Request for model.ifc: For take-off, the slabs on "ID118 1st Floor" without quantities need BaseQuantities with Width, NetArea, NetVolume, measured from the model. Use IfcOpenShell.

First a look at what the model holds.

```python
import ifcopenshell
import ifcopenshell.util.element
import ifcopenshell.util.unit

model = ifcopenshell.open("model.ifc")
print(model.schema)
for unit_type in ("LENGTHUNIT", "AREAUNIT", "VOLUMEUNIT"):
    print(unit_type, ifcopenshell.util.unit.calculate_unit_scale(model, unit_type))
storey = next(s for s in model.by_type("IfcBuildingStorey") if s.Name == "ID118 1st Floor")
slabs = [e for e in ifcopenshell.util.element.get_decomposition(storey) if e.is_a("IfcSlab")]
for e in sorted(slabs, key=lambda e: e.id()):
    print(e.id(), e.is_a(), e.Name, list(ifcopenshell.util.element.get_psets(e, qtos_only=True)), sep=" | ")
```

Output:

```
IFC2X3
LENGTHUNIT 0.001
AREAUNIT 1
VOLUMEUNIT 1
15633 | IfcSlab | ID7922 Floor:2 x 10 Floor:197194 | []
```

```python
import ifcopenshell
import ifcopenshell.api.pset
import ifcopenshell.geom
import ifcopenshell.util.element
import ifcopenshell.util.shape
import ifcopenshell.util.unit

model = ifcopenshell.open("model.ifc")
unit_scale = ifcopenshell.util.unit.calculate_unit_scale(model)
area_scale = ifcopenshell.util.unit.calculate_unit_scale(model, "AREAUNIT")
volume_scale = ifcopenshell.util.unit.calculate_unit_scale(model, "VOLUMEUNIT")
settings = ifcopenshell.geom.settings()

storey = next(s for s in model.by_type("IfcBuildingStorey") if s.Name == "ID118 1st Floor")
slabs = [e for e in ifcopenshell.util.element.get_decomposition(storey) if e.is_a("IfcSlab")]

for e in sorted(slabs, key=lambda e: e.id()):
    if ifcopenshell.util.element.get_psets(e, qtos_only=True, should_inherit=False):
        continue
    # Geometry comes back in metres, in the element's own axes.
    shape = ifcopenshell.geom.create_shape(settings, e)
    values = {
        "Width": ifcopenshell.util.shape.get_z(shape.geometry) / unit_scale,
        "NetArea": ifcopenshell.util.shape.get_footprint_area(shape.geometry) / area_scale,
        "NetVolume": ifcopenshell.util.shape.get_volume(shape.geometry) / volume_scale,
    }
    qto = ifcopenshell.api.pset.add_qto(model, product=e, name="BaseQuantities")
    ifcopenshell.api.pset.edit_qto(model, qto=qto, properties=values)
    print(e.id(), {k: round(v, 3) for k, v in values.items()})

model.write("model-out.ifc")
```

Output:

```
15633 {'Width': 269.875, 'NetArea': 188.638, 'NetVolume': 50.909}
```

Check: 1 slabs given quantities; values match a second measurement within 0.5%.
